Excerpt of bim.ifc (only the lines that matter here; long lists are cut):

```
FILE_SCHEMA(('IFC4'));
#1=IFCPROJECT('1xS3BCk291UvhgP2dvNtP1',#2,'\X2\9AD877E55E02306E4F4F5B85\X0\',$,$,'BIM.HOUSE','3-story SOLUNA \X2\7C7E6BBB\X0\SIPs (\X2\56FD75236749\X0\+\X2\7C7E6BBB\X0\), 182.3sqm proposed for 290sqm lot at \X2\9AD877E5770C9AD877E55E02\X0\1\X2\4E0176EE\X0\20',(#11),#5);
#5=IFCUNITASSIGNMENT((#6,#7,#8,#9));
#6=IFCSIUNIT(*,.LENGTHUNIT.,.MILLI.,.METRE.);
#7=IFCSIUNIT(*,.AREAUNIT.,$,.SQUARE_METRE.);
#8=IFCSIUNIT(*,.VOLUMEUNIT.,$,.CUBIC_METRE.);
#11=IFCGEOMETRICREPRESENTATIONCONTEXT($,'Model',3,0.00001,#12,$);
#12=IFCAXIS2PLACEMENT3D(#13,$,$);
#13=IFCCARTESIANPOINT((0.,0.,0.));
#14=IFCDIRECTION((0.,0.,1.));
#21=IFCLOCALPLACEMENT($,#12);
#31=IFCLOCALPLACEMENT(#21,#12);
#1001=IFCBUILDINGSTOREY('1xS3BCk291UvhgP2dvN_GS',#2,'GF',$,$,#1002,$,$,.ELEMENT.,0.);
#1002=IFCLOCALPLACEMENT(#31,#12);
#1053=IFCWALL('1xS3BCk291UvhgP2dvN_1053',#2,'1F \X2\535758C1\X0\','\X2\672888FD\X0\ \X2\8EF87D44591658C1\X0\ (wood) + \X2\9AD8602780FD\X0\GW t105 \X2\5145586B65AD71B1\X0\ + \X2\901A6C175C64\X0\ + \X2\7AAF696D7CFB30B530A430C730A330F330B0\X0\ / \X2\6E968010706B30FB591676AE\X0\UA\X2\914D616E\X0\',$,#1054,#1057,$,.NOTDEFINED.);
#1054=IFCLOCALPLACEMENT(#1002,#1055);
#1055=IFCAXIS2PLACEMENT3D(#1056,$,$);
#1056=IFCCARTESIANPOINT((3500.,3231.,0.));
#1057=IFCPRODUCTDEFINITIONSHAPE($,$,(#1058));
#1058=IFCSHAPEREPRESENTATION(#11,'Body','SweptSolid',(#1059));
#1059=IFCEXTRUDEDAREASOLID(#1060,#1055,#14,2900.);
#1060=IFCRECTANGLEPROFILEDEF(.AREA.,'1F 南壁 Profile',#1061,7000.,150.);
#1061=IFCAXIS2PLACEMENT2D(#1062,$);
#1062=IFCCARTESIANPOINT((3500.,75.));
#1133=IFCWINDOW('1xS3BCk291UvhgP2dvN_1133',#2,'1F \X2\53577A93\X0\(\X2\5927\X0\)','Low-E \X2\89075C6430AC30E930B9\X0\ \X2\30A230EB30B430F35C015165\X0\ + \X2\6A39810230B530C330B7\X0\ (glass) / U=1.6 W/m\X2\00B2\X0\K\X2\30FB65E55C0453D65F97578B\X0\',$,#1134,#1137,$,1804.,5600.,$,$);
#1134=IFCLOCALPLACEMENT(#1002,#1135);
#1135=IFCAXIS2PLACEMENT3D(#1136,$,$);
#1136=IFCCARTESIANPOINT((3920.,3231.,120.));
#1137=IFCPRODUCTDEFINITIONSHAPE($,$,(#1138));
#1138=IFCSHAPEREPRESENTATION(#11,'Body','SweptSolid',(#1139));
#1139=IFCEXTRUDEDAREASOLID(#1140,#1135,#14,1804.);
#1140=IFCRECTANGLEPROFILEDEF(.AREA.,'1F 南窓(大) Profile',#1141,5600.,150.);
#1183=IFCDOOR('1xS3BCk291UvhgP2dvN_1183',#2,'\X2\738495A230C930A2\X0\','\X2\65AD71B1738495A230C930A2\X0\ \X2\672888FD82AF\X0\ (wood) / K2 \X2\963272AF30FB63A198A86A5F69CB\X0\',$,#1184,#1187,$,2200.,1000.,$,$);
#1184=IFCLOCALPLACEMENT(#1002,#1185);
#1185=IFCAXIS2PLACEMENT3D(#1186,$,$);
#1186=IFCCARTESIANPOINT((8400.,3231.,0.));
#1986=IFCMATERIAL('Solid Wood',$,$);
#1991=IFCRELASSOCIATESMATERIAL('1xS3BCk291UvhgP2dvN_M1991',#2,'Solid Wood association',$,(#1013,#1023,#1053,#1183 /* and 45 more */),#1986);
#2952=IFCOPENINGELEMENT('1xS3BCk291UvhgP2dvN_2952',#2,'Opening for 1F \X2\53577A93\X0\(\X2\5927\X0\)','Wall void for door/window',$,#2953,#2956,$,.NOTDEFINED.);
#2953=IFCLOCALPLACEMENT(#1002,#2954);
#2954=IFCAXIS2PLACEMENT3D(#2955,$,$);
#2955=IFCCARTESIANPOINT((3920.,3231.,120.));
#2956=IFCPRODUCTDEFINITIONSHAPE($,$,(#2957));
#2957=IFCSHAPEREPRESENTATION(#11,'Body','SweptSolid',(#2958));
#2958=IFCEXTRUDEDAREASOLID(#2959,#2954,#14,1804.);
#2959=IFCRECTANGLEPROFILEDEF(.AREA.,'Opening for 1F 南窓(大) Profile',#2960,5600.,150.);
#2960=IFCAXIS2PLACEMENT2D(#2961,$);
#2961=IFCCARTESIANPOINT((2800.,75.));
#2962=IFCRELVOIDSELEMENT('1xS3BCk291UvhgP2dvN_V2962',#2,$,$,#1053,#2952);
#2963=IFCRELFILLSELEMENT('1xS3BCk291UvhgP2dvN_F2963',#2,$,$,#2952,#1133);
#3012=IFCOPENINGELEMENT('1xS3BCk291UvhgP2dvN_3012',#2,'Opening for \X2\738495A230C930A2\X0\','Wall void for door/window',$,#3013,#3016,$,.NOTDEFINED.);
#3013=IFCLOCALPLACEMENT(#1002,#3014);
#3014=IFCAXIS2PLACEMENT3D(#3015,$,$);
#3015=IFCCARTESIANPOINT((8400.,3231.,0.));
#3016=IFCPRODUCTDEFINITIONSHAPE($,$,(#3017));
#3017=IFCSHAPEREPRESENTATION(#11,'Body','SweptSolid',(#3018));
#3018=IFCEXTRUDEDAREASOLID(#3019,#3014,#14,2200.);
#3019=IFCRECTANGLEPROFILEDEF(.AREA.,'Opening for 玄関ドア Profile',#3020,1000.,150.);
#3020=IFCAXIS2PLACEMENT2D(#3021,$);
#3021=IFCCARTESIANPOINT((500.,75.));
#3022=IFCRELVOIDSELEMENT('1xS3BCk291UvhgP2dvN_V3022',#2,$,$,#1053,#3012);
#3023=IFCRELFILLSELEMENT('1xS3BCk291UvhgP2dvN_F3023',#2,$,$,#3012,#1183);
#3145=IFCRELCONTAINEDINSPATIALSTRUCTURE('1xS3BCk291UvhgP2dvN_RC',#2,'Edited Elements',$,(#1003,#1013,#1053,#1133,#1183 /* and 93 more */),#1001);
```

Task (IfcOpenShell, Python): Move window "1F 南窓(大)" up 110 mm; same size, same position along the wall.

```python
import numpy as np
import ifcopenshell
import ifcopenshell.api.geometry
import ifcopenshell.util.placement
import ifcopenshell.util.unit

model = ifcopenshell.open("bim.ifc")
unit_scale = ifcopenshell.util.unit.calculate_unit_scale(model)

window = model.by_guid("1xS3BCk291UvhgP2dvN_1133")
opening = window.FillsVoids[0].RelatingOpeningElement
dz = 0.11 / unit_scale

shift = np.array([0.0, 0.0, dz])
# The window is not placed relative to its opening, so move both.
for product in (opening, window):
    matrix = ifcopenshell.util.placement.get_local_placement(product.ObjectPlacement)
    matrix[:3, 3] += shift
    ifcopenshell.api.geometry.edit_object_placement(model, product=product, matrix=matrix, is_si=False)

print(f"moved by {dz * unit_scale:+.3f} m")

model.write("bim_rev.ifc")
```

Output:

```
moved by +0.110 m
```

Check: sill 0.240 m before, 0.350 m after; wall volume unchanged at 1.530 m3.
